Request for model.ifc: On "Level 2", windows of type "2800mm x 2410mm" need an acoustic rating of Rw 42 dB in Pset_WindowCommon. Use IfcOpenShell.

First a look at what the model holds.

```python
import ifcopenshell
import ifcopenshell.util.element

model = ifcopenshell.open("model.ifc")
print(model.schema)
storey = next(s for s in model.by_type("IfcBuildingStorey") if s.Name == "Level 2")
windows = [e for e in ifcopenshell.util.element.get_decomposition(storey) if e.is_a("IfcWindow")]
seen = {}
for e in windows:
    element_type = ifcopenshell.util.element.get_type(e)
    key = (element_type.Name if element_type != e and element_type else None, ifcopenshell.util.element.get_pset(e, "Pset_WindowCommon", "AcousticRating"))
    seen[key] = seen.get(key, 0) + 1
for (name, value), count in sorted(seen.items(), key=str):
    print(count, "x", name, "|", value)
```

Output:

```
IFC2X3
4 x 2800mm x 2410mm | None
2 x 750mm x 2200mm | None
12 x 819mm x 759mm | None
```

```python
import ifcopenshell
import ifcopenshell.api.pset
import ifcopenshell.util.element

model = ifcopenshell.open("model.ifc")

storey = next(s for s in model.by_type("IfcBuildingStorey") if s.Name == "Level 2")
windows = [e for e in ifcopenshell.util.element.get_decomposition(storey) if e.is_a("IfcWindow")]

count = 0
for e in windows:
    element_type = ifcopenshell.util.element.get_type(e)
    if element_type in (None, e) or element_type.Name != "2800mm x 2410mm":
        continue
    # add_pset returns the element's existing set when there is one.
    pset = ifcopenshell.api.pset.add_pset(model, product=e, name="Pset_WindowCommon")
    ifcopenshell.api.pset.edit_pset(model, pset=pset, properties={"AcousticRating": "Rw 42 dB"})
    count += 1

print(count, "windows updated")

model.write("model_v2.ifc")
```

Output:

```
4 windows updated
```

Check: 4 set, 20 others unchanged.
